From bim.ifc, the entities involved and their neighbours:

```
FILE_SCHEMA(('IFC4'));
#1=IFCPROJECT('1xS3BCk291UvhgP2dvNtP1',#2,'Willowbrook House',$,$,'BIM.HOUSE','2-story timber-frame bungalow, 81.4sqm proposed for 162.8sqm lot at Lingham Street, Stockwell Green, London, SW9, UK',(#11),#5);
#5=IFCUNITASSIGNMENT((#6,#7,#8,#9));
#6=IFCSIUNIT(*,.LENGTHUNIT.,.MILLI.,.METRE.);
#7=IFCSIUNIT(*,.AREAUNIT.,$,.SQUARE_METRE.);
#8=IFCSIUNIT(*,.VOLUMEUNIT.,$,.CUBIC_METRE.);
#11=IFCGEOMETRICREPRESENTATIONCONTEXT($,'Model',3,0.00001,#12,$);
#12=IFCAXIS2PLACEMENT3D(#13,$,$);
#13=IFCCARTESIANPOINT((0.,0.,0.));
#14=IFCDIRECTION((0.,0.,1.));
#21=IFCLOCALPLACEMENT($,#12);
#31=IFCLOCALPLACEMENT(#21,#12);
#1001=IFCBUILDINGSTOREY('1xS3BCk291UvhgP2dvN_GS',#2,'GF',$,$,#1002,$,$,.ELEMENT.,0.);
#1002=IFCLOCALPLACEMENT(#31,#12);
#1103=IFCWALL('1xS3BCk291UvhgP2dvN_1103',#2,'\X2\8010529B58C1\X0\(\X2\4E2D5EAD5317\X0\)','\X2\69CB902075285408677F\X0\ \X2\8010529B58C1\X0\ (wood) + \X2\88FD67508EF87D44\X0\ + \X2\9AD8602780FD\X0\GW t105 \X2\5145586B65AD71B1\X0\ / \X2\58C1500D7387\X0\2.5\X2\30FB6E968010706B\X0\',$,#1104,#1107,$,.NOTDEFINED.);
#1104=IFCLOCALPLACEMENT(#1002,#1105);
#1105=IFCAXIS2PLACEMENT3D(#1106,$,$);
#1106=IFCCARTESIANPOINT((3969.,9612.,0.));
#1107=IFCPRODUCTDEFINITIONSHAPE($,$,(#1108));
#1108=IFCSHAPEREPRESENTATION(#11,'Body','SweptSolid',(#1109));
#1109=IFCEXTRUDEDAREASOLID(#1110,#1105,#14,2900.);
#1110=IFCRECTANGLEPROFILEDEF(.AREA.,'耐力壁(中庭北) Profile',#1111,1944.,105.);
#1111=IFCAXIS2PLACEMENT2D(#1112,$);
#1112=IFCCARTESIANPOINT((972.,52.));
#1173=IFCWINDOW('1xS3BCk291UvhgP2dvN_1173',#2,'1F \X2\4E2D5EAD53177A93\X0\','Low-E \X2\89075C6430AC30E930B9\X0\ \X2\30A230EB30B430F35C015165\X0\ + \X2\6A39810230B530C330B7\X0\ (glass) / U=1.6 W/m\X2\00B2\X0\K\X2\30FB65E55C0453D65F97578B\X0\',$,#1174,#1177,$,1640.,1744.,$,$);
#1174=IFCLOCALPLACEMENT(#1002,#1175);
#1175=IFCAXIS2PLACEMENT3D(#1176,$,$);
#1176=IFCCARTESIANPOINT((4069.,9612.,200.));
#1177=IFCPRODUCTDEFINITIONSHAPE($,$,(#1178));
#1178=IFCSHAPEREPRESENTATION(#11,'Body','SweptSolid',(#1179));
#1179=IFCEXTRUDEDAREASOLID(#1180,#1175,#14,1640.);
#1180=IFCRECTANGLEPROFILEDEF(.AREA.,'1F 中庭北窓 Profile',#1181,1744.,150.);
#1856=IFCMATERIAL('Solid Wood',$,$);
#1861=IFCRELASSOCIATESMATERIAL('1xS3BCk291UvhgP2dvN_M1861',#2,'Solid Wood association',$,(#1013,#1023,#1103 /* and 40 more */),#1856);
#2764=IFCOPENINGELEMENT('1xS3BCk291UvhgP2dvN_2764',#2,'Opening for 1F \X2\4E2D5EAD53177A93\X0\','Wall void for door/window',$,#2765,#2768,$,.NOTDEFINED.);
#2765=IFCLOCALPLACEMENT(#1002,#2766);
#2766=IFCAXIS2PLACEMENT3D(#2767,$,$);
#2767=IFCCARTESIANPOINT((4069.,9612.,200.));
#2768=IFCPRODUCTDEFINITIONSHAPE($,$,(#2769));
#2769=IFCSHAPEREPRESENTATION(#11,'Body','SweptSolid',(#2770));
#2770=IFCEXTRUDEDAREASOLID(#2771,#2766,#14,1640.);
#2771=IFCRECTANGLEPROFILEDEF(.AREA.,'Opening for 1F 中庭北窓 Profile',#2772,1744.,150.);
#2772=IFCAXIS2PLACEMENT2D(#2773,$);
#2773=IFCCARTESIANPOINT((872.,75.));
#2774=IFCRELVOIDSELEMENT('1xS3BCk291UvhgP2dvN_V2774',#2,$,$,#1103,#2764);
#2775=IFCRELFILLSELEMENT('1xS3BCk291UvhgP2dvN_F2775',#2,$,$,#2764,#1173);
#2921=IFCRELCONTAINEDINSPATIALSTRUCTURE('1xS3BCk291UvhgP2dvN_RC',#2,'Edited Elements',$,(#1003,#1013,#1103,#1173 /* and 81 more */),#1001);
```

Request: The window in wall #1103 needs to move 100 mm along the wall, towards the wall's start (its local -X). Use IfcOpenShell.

```python
import ifcopenshell
import ifcopenshell.api.geometry
import ifcopenshell.util.placement
import ifcopenshell.util.unit

model = ifcopenshell.open("bim.ifc")
unit_scale = ifcopenshell.util.unit.calculate_unit_scale(model)

window = model.by_guid("1xS3BCk291UvhgP2dvN_1173")
opening = window.FillsVoids[0].RelatingOpeningElement
wall = opening.VoidsElements[0].RelatingBuildingElement

wall_matrix = ifcopenshell.util.placement.get_local_placement(wall.ObjectPlacement)
shift = wall_matrix[:3, 0] * -0.1 / unit_scale
before = ifcopenshell.util.placement.get_local_placement(window.ObjectPlacement)[:3, 3].copy()

# The window is not placed relative to its opening, so move both.
for product in (opening, window):
    matrix = ifcopenshell.util.placement.get_local_placement(product.ObjectPlacement)
    matrix[:3, 3] += shift
    ifcopenshell.api.geometry.edit_object_placement(model, product=product, matrix=matrix, is_si=False)

after = ifcopenshell.util.placement.get_local_placement(window.ObjectPlacement)[:3, 3]
print("window moved by", (after - before).round(3) + 0.0)

model.write("bim_updated.ifc")
```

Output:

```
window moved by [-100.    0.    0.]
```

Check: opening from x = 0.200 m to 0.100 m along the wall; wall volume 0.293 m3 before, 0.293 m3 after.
